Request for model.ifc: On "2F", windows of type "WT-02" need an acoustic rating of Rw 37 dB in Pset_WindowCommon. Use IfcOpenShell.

First a look at what the model holds.

```python
import ifcopenshell
import ifcopenshell.util.element

model = ifcopenshell.open("model.ifc")
print(model.schema)
storey = next(s for s in model.by_type("IfcBuildingStorey") if s.Name == "2F")
windows = [e for e in ifcopenshell.util.element.get_decomposition(storey) if e.is_a("IfcWindow")]
seen = {}
for e in windows:
    element_type = ifcopenshell.util.element.get_type(e)
    key = (element_type.Name if element_type != e and element_type else None, ifcopenshell.util.element.get_pset(e, "Pset_WindowCommon", "AcousticRating"))
    seen[key] = seen.get(key, 0) + 1
for (name, value), count in sorted(seen.items(), key=str):
    print(count, "x", name, "|", value)
```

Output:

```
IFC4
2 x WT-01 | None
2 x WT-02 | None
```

```python
import ifcopenshell
import ifcopenshell.api.pset
import ifcopenshell.util.element

model = ifcopenshell.open("model.ifc")

storey = next(s for s in model.by_type("IfcBuildingStorey") if s.Name == "2F")
windows = [e for e in ifcopenshell.util.element.get_decomposition(storey) if e.is_a("IfcWindow")]

count = 0
for e in windows:
    element_type = ifcopenshell.util.element.get_type(e)
    if element_type in (None, e) or element_type.Name != "WT-02":
        continue
    # add_pset returns the element's existing set when there is one.
    pset = ifcopenshell.api.pset.add_pset(model, product=e, name="Pset_WindowCommon")
    ifcopenshell.api.pset.edit_pset(model, pset=pset, properties={"AcousticRating": "Rw 37 dB"})
    count += 1

print(count, "windows updated")

model.write("model_rev.ifc")
```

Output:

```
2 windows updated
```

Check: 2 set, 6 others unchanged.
